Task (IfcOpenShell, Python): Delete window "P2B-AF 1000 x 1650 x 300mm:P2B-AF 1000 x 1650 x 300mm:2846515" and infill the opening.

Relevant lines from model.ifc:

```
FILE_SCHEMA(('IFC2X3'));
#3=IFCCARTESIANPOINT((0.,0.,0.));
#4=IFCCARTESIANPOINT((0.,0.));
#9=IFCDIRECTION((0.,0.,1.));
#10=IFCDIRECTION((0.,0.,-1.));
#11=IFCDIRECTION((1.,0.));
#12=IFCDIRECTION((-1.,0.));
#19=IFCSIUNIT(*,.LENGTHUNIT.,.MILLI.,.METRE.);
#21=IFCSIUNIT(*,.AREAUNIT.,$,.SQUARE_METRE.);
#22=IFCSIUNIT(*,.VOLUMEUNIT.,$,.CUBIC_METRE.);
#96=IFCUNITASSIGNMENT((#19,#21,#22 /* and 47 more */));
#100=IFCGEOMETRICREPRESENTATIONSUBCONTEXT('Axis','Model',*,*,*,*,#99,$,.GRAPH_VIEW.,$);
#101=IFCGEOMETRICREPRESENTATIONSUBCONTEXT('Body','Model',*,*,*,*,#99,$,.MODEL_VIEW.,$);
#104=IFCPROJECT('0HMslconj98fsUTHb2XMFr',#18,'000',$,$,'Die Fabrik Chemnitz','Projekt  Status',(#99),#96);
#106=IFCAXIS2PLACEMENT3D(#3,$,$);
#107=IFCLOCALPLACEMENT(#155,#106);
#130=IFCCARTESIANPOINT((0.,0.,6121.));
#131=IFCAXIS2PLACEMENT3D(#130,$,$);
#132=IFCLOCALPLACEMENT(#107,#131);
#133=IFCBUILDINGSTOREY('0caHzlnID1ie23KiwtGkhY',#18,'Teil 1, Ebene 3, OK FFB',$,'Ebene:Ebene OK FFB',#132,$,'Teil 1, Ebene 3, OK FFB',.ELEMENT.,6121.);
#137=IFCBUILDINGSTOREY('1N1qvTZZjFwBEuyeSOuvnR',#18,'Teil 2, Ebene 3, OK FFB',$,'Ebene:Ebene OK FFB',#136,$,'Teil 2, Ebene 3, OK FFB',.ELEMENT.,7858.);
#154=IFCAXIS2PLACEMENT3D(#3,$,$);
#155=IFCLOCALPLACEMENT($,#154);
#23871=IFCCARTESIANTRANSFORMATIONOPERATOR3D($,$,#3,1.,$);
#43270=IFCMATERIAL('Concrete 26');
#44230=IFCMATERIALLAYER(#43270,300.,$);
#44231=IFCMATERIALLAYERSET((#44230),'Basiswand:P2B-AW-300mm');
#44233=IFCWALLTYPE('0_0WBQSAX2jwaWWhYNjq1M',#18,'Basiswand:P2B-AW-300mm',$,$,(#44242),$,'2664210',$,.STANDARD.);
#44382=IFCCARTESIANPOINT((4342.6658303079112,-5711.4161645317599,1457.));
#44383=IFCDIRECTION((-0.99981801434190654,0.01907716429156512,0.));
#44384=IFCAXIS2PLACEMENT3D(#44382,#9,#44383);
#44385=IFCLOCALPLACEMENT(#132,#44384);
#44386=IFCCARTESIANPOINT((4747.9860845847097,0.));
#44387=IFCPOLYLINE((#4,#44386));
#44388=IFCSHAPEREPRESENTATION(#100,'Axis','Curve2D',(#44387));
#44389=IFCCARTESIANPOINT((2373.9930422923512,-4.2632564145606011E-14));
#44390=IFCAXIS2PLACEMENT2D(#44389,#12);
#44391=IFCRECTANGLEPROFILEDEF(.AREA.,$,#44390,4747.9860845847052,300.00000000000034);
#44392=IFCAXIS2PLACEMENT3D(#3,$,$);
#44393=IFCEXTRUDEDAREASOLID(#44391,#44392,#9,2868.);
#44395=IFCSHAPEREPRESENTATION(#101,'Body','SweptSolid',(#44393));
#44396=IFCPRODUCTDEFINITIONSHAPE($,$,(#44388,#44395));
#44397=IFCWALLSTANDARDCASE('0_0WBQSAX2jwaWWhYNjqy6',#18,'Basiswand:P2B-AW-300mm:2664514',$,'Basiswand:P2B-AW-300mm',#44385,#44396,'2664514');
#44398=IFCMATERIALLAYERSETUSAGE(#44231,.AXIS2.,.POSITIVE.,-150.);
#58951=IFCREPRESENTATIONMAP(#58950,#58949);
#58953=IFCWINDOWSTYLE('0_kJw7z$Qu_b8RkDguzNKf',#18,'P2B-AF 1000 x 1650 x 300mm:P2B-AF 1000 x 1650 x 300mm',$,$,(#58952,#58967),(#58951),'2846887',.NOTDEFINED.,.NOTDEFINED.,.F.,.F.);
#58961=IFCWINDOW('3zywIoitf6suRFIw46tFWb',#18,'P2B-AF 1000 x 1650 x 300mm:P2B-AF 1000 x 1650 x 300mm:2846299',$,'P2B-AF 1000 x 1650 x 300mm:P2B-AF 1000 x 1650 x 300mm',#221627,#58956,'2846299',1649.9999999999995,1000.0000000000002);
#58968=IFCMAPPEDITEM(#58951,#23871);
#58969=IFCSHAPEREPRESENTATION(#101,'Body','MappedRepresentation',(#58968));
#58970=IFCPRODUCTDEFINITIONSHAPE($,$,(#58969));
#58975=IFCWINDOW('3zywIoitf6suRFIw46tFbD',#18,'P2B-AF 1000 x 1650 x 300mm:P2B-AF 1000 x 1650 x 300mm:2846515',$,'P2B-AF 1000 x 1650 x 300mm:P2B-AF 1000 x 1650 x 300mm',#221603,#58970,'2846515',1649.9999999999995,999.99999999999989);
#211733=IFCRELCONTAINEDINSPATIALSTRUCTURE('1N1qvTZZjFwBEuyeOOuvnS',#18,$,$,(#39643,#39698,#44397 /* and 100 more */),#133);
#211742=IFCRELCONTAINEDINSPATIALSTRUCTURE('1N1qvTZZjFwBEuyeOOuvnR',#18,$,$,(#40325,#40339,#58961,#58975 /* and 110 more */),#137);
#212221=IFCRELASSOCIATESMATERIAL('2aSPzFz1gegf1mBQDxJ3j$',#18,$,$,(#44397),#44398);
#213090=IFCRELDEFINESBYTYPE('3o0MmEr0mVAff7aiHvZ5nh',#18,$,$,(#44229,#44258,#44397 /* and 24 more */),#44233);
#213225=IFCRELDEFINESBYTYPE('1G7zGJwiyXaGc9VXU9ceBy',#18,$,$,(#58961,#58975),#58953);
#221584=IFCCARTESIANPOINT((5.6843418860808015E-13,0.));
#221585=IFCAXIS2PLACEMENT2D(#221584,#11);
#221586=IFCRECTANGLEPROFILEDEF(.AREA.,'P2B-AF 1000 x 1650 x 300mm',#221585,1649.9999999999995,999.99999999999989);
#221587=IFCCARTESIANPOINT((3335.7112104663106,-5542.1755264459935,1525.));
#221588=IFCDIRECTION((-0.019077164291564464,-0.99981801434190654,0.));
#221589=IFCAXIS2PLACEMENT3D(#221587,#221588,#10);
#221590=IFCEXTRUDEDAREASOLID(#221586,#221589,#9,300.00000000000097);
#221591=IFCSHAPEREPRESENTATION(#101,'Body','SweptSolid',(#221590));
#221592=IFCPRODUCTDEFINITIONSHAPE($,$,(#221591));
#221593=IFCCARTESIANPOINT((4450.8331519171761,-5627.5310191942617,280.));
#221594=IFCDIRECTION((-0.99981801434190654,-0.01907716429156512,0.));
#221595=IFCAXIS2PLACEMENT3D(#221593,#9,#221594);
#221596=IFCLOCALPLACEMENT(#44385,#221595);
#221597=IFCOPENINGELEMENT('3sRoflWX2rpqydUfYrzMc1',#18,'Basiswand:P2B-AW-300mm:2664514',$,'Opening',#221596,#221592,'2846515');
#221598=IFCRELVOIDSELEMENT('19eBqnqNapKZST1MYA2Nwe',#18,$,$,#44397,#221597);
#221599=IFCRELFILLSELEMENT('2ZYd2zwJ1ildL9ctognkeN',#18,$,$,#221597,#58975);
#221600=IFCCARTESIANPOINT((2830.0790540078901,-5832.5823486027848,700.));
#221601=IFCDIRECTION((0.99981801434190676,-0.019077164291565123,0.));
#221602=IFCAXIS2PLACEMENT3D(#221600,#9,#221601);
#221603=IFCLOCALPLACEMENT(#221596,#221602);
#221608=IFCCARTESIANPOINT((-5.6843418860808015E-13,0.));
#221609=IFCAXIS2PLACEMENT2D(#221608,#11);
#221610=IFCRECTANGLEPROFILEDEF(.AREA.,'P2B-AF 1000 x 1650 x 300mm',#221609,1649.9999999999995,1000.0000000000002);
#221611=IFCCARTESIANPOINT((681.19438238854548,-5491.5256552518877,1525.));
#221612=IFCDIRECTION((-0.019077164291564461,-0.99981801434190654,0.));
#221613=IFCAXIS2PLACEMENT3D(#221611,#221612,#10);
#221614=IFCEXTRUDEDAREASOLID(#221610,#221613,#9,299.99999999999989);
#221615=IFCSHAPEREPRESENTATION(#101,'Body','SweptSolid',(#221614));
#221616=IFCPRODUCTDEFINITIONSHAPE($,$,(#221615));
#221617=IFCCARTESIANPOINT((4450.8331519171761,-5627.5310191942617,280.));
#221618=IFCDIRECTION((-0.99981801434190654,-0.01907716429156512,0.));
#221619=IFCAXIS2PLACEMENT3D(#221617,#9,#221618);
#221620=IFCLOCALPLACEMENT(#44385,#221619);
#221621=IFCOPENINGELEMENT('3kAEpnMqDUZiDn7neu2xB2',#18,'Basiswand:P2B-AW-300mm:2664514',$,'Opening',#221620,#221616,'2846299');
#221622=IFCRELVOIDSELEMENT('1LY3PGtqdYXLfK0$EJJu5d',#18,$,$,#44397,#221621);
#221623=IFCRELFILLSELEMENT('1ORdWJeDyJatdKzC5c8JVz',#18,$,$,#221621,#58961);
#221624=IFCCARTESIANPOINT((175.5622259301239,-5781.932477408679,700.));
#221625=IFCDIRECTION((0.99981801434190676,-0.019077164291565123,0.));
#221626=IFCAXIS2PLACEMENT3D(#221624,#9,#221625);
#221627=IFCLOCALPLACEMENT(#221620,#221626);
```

```python
import ifcopenshell
import ifcopenshell.api.feature
import ifcopenshell.api.root
import ifcopenshell.geom
import ifcopenshell.util.shape

model = ifcopenshell.open("model.ifc")
settings = ifcopenshell.geom.settings()


def volume(element):
    """Net volume in cubic metres, openings subtracted."""
    shape = ifcopenshell.geom.create_shape(settings, element)
    return ifcopenshell.util.shape.get_volume(shape.geometry)


window = model.by_id(58975)
opening = window.FillsVoids[0].RelatingOpeningElement
wall = opening.VoidsElements[0].RelatingBuildingElement
before = volume(wall)

ifcopenshell.api.root.remove_product(model, product=window)
ifcopenshell.api.feature.remove_feature(model, feature=opening)

after = volume(wall)

print(f"wall volume {before:.3f} -> {after:.3f} m3")

model.write("model_updated.ifc")
```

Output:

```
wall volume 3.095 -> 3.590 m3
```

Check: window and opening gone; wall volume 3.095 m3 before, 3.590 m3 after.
